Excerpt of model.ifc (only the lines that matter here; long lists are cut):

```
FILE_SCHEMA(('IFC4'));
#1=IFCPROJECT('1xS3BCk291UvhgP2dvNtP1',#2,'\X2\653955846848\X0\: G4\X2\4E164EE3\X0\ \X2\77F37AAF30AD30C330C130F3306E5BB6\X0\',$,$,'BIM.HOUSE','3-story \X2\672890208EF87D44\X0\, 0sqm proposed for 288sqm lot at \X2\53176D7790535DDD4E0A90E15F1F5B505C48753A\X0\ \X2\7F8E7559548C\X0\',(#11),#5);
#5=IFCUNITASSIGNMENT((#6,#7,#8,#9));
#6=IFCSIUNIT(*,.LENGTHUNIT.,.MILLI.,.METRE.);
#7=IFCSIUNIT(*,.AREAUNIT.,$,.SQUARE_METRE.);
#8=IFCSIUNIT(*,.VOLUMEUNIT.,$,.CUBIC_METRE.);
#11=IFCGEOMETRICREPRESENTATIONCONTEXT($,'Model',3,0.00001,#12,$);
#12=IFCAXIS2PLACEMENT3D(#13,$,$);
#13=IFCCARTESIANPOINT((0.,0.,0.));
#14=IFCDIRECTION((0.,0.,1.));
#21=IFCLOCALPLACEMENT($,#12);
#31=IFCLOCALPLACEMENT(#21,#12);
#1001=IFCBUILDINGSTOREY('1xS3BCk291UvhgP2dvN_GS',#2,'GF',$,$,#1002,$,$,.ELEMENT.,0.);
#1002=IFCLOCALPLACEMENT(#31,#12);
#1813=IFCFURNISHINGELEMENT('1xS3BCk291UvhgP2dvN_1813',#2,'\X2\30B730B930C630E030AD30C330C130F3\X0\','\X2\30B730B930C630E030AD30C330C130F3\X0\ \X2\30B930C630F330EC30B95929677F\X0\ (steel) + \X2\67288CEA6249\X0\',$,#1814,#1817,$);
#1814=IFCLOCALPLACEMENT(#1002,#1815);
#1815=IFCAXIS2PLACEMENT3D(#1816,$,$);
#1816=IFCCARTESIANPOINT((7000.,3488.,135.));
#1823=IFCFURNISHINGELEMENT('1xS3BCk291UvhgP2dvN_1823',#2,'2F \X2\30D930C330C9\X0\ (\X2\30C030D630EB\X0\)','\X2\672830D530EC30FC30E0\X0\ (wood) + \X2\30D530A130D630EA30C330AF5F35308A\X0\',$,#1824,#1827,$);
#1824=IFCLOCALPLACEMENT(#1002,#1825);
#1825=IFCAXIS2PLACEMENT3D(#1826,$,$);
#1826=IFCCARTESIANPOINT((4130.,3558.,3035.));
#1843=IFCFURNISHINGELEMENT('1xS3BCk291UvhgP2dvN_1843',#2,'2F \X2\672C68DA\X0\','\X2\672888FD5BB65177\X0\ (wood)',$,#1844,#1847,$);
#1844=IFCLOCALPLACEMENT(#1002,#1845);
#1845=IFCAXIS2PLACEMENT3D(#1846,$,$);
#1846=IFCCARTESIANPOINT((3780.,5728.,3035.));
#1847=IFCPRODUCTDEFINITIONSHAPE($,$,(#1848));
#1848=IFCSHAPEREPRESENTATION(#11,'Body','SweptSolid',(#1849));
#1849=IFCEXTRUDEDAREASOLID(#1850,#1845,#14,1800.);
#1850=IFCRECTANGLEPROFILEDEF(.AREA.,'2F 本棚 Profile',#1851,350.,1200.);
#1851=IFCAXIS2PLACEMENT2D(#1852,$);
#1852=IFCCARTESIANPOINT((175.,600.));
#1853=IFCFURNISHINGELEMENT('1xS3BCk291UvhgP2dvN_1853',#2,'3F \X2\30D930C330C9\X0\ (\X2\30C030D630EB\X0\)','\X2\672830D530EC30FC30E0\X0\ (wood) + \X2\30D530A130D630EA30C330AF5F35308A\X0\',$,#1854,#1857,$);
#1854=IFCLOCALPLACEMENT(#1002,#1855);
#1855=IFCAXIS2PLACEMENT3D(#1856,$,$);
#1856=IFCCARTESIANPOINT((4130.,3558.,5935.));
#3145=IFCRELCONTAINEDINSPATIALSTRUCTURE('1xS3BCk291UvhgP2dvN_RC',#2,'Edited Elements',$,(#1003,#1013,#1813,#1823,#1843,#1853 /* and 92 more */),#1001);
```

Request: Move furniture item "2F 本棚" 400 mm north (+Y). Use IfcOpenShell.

```python
import ifcopenshell
import ifcopenshell.api.geometry
import ifcopenshell.util.placement

model = ifcopenshell.open("model.ifc")

item = model.by_guid("1xS3BCk291UvhgP2dvN_1843")
matrix = ifcopenshell.util.placement.get_local_placement(item.ObjectPlacement)
matrix[1, 3] += 400.0
ifcopenshell.api.geometry.edit_object_placement(model, product=item, matrix=matrix, is_si=False)

print(ifcopenshell.util.placement.get_local_placement(item.ObjectPlacement).round(3) + 0.0)

model.write("model_edited.ifc")
```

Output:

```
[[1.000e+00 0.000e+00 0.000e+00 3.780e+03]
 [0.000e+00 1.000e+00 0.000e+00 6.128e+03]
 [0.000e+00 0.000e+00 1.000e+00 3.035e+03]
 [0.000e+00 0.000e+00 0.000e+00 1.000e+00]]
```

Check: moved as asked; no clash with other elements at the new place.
